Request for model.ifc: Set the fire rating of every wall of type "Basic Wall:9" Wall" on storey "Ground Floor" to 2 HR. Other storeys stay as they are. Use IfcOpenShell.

First a look at what the model holds.

```python
import ifcopenshell
import ifcopenshell.util.element

model = ifcopenshell.open("model.ifc")
print(model.schema)
storey = next(s for s in model.by_type("IfcBuildingStorey") if s.Name == "Ground Floor")
walls = [e for e in ifcopenshell.util.element.get_decomposition(storey) if e.is_a("IfcWall")]
seen = {}
for e in walls:
    element_type = ifcopenshell.util.element.get_type(e)
    key = (element_type.Name if element_type != e and element_type else None, ifcopenshell.util.element.get_pset(e, "Pset_WallCommon", "FireRating"))
    seen[key] = seen.get(key, 0) + 1
for (name, value), count in sorted(seen.items(), key=str):
    print(count, "x", name, "|", value)
```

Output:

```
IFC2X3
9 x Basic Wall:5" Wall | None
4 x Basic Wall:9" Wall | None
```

```python
import ifcopenshell
import ifcopenshell.api.pset
import ifcopenshell.util.element

model = ifcopenshell.open("model.ifc")

storey = next(s for s in model.by_type("IfcBuildingStorey") if s.Name == "Ground Floor")
walls = [e for e in ifcopenshell.util.element.get_decomposition(storey) if e.is_a("IfcWall")]

count = 0
for e in walls:
    element_type = ifcopenshell.util.element.get_type(e)
    if element_type in (None, e) or element_type.Name != 'Basic Wall:9" Wall':
        continue
    # add_pset returns the element's existing set when there is one.
    pset = ifcopenshell.api.pset.add_pset(model, product=e, name="Pset_WallCommon")
    ifcopenshell.api.pset.edit_pset(model, pset=pset, properties={"FireRating": "2 HR"})
    count += 1

print(count, "walls updated")

model.write("model_edited.ifc")
```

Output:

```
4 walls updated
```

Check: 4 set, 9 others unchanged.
